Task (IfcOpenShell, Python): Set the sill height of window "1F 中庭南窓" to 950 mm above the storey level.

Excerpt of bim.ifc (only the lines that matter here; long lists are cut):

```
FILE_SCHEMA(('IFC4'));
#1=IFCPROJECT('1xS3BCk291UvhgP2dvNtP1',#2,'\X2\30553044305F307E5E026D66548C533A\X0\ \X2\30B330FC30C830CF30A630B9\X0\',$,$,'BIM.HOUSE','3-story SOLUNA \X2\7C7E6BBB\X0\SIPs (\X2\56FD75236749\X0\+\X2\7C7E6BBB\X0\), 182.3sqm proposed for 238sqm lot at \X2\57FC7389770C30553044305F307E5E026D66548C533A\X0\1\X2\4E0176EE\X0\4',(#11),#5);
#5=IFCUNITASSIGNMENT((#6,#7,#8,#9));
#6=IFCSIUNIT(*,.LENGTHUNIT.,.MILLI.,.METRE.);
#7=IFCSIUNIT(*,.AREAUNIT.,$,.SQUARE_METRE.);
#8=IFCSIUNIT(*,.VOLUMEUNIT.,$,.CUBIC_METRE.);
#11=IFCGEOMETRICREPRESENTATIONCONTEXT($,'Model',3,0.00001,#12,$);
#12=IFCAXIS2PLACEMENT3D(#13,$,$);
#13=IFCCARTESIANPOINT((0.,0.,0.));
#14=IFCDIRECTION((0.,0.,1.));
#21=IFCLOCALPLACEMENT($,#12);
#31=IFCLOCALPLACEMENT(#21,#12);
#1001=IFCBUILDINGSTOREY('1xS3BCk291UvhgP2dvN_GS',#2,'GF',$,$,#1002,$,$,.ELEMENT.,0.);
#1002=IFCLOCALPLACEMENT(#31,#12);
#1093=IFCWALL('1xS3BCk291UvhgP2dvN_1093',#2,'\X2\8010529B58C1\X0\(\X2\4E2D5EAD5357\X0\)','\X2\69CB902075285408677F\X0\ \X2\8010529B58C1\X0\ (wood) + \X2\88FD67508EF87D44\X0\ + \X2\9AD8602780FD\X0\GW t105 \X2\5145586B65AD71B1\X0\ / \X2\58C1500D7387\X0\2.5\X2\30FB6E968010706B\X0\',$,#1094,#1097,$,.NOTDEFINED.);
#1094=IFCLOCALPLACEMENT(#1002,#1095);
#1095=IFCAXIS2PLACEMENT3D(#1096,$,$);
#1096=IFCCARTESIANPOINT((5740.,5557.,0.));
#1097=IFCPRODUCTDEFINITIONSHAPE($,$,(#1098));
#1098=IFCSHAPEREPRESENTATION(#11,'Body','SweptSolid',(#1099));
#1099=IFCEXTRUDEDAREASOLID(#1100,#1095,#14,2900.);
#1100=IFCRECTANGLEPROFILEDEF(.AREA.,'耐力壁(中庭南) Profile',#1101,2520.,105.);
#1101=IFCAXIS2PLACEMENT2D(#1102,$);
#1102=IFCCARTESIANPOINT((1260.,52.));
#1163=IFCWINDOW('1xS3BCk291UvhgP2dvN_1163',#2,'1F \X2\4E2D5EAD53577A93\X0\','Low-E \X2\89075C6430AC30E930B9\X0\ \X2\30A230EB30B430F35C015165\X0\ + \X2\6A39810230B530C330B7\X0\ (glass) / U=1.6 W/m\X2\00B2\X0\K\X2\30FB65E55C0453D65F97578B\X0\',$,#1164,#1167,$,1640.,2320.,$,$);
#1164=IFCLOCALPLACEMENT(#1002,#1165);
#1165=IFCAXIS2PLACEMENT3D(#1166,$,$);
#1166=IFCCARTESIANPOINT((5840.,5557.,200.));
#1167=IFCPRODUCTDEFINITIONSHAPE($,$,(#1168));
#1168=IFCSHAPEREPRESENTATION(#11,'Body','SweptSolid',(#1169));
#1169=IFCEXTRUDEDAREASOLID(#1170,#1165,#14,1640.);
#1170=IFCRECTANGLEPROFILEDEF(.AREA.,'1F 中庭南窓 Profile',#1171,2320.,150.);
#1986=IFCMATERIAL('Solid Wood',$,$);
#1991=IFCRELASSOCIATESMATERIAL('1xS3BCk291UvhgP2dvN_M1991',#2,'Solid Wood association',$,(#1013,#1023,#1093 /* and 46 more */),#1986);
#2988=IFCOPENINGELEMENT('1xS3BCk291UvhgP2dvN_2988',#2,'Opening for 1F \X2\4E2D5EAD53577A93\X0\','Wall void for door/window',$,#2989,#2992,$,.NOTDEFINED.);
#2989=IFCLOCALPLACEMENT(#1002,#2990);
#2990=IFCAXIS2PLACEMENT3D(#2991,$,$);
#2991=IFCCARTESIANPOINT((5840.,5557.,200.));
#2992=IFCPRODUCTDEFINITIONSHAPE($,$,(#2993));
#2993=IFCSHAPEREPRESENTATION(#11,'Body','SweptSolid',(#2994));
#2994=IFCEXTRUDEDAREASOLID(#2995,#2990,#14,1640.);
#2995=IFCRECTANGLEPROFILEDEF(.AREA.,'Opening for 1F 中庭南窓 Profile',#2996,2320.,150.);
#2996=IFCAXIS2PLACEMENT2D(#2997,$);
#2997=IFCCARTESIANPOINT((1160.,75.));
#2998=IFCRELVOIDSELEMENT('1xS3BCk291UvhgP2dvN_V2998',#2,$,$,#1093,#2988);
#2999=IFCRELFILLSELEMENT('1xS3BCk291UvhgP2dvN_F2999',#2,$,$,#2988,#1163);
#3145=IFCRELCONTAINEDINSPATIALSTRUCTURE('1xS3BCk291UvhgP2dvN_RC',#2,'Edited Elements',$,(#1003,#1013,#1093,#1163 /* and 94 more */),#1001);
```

```python
import numpy as np
import ifcopenshell
import ifcopenshell.api.geometry
import ifcopenshell.geom
import ifcopenshell.util.element
import ifcopenshell.util.placement
import ifcopenshell.util.shape
import ifcopenshell.util.unit

model = ifcopenshell.open("bim.ifc")
unit_scale = ifcopenshell.util.unit.calculate_unit_scale(model)

window = model.by_guid("1xS3BCk291UvhgP2dvN_1163")
opening = window.FillsVoids[0].RelatingOpeningElement
storey = ifcopenshell.util.element.get_container(window, ifc_class="IfcBuildingStorey")
level = ifcopenshell.util.placement.get_local_placement(storey.ObjectPlacement)[2, 3]

# The opening's origin need not be at the sill, so measure its lowest point.
shape = ifcopenshell.geom.create_shape(ifcopenshell.geom.settings(), opening)
bottom = ifcopenshell.util.shape.get_shape_bottom_elevation(shape, shape.geometry) / unit_scale
dz = level + 950.0 - bottom

shift = np.array([0.0, 0.0, dz])
# The window is not placed relative to its opening, so move both.
for product in (opening, window):
    matrix = ifcopenshell.util.placement.get_local_placement(product.ObjectPlacement)
    matrix[:3, 3] += shift
    ifcopenshell.api.geometry.edit_object_placement(model, product=product, matrix=matrix, is_si=False)

print(f"moved by {dz * unit_scale:+.3f} m")

model.write("bim-out.ifc")
```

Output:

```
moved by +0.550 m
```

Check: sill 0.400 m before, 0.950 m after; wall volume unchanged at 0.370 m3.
